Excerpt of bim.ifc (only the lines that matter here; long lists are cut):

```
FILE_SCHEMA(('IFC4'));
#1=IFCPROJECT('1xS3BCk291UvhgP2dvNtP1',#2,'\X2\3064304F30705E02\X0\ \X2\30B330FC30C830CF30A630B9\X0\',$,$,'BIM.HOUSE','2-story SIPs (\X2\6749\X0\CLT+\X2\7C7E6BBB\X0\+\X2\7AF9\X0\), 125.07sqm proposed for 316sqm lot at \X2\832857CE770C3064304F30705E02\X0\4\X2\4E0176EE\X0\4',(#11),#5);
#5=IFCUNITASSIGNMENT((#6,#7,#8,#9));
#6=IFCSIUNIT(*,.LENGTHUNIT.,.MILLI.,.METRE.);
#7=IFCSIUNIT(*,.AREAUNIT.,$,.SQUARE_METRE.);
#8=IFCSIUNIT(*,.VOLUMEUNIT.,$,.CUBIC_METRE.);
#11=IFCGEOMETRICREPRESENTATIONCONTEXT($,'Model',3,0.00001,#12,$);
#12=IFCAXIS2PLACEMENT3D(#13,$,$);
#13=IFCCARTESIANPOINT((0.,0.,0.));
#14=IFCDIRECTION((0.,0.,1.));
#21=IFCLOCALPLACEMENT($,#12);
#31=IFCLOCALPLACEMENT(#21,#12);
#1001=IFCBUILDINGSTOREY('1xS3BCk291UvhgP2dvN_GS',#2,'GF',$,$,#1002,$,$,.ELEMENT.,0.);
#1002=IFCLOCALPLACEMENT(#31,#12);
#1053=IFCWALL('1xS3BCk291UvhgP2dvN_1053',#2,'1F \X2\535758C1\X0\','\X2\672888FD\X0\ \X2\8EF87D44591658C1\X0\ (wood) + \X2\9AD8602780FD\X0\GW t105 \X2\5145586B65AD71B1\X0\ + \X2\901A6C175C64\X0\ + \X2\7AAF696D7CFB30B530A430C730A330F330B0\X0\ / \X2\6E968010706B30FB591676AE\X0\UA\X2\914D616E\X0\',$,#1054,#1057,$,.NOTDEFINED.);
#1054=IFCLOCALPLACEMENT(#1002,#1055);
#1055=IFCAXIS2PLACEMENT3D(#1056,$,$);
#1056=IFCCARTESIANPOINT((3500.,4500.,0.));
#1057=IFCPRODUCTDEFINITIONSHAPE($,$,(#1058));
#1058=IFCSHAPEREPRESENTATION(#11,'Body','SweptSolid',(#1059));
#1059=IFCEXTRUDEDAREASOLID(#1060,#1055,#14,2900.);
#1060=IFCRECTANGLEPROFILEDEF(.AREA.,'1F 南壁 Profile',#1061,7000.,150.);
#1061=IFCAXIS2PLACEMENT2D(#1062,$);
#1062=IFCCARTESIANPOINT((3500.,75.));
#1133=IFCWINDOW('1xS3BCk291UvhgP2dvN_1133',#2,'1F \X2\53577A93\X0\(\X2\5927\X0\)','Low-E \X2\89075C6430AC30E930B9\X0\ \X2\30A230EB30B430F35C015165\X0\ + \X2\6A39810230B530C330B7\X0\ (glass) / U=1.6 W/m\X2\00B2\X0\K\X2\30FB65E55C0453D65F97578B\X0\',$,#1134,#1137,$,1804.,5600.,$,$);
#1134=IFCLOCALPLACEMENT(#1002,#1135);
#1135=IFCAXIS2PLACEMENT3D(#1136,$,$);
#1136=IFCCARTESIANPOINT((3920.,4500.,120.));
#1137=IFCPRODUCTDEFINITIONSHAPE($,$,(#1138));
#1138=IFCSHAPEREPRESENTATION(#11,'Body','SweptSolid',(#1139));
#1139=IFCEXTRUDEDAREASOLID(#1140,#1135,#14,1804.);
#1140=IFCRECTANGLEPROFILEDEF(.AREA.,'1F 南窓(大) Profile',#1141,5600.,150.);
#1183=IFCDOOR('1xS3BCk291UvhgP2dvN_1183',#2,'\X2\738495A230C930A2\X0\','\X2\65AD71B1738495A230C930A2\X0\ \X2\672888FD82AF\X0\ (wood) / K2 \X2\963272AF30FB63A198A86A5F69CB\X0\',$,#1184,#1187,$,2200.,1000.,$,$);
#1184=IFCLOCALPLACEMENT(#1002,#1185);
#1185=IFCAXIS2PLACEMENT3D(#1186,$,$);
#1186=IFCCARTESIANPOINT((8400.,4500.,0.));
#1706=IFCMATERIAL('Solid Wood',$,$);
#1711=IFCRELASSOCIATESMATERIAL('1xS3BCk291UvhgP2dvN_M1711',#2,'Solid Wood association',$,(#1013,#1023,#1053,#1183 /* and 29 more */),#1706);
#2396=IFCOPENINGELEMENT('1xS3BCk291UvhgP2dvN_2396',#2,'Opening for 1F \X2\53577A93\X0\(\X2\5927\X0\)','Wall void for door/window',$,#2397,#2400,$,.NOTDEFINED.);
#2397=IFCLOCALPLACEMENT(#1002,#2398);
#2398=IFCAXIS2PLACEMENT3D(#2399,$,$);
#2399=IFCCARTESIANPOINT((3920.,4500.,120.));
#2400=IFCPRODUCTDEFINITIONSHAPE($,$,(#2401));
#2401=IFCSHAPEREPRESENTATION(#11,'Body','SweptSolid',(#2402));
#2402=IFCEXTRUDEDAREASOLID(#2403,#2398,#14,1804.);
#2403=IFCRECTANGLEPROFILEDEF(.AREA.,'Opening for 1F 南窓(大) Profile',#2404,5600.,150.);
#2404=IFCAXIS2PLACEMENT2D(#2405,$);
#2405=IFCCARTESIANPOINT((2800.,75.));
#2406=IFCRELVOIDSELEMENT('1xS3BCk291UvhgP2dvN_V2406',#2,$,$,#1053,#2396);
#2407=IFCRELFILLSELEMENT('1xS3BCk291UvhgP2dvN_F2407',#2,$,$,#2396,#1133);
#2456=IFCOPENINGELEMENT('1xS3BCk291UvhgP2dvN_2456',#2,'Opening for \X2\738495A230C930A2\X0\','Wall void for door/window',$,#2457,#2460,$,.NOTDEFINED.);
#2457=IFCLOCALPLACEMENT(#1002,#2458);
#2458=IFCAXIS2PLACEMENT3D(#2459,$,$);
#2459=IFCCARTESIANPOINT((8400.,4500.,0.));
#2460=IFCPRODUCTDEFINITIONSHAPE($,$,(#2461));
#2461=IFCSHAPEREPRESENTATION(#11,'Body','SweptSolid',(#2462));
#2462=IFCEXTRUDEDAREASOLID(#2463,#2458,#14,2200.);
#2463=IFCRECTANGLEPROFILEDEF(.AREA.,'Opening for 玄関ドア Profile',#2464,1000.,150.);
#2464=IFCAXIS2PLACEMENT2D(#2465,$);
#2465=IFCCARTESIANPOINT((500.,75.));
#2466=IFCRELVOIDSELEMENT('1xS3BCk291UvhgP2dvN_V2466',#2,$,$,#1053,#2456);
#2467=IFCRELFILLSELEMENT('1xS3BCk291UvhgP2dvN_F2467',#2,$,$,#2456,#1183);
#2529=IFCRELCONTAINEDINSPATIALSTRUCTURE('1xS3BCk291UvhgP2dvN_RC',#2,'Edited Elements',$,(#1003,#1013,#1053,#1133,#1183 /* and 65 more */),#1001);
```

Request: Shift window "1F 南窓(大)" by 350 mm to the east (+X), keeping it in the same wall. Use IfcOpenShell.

```python
import ifcopenshell
import ifcopenshell.api.geometry
import ifcopenshell.util.placement
import ifcopenshell.util.unit

model = ifcopenshell.open("bim.ifc")
unit_scale = ifcopenshell.util.unit.calculate_unit_scale(model)

window = model.by_id(1133)
opening = window.FillsVoids[0].RelatingOpeningElement
wall = opening.VoidsElements[0].RelatingBuildingElement

wall_matrix = ifcopenshell.util.placement.get_local_placement(wall.ObjectPlacement)
shift = wall_matrix[:3, 0] * 0.35 / unit_scale
before = ifcopenshell.util.placement.get_local_placement(window.ObjectPlacement)[:3, 3].copy()

# The window is not placed relative to its opening, so move both.
for product in (opening, window):
    matrix = ifcopenshell.util.placement.get_local_placement(product.ObjectPlacement)
    matrix[:3, 3] += shift
    ifcopenshell.api.geometry.edit_object_placement(model, product=product, matrix=matrix, is_si=False)

after = ifcopenshell.util.placement.get_local_placement(window.ObjectPlacement)[:3, 3]
print("window moved by", (after - before).round(3) + 0.0)

model.write("bim-out.ifc")
```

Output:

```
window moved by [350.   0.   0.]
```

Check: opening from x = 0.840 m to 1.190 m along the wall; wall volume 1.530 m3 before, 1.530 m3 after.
